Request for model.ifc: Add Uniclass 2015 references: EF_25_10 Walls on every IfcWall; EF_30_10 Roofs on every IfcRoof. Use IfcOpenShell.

First a look at what the model holds.

```python
import ifcopenshell

model = ifcopenshell.open("model.ifc")
print(model.schema)
print("classifications:", [c.Name for c in model.by_type("IfcClassification")])
for ifc_class in ("IfcDoor", "IfcRoof", "IfcStair", "IfcWall", "IfcWindow"):
    print(ifc_class, len(model.by_type(ifc_class)))
```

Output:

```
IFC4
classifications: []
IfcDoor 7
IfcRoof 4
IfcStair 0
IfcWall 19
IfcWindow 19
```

```python
import ifcopenshell
import ifcopenshell.api.classification

model = ifcopenshell.open("model.ifc")

system = ifcopenshell.api.classification.add_classification(model, classification="Uniclass 2015")

codes = {
    "IfcWall": ("EF_25_10", "Walls"),
    "IfcRoof": ("EF_30_10", "Roofs"),
}
for ifc_class, (code, name) in codes.items():
    products = model.by_type(ifc_class)
    ifcopenshell.api.classification.add_reference(
        model, products=products, classification=system, identification=code, name=name
    )
    print(code, len(products))

model.write("model_updated.ifc")
```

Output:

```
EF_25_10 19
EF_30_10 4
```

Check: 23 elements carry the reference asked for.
